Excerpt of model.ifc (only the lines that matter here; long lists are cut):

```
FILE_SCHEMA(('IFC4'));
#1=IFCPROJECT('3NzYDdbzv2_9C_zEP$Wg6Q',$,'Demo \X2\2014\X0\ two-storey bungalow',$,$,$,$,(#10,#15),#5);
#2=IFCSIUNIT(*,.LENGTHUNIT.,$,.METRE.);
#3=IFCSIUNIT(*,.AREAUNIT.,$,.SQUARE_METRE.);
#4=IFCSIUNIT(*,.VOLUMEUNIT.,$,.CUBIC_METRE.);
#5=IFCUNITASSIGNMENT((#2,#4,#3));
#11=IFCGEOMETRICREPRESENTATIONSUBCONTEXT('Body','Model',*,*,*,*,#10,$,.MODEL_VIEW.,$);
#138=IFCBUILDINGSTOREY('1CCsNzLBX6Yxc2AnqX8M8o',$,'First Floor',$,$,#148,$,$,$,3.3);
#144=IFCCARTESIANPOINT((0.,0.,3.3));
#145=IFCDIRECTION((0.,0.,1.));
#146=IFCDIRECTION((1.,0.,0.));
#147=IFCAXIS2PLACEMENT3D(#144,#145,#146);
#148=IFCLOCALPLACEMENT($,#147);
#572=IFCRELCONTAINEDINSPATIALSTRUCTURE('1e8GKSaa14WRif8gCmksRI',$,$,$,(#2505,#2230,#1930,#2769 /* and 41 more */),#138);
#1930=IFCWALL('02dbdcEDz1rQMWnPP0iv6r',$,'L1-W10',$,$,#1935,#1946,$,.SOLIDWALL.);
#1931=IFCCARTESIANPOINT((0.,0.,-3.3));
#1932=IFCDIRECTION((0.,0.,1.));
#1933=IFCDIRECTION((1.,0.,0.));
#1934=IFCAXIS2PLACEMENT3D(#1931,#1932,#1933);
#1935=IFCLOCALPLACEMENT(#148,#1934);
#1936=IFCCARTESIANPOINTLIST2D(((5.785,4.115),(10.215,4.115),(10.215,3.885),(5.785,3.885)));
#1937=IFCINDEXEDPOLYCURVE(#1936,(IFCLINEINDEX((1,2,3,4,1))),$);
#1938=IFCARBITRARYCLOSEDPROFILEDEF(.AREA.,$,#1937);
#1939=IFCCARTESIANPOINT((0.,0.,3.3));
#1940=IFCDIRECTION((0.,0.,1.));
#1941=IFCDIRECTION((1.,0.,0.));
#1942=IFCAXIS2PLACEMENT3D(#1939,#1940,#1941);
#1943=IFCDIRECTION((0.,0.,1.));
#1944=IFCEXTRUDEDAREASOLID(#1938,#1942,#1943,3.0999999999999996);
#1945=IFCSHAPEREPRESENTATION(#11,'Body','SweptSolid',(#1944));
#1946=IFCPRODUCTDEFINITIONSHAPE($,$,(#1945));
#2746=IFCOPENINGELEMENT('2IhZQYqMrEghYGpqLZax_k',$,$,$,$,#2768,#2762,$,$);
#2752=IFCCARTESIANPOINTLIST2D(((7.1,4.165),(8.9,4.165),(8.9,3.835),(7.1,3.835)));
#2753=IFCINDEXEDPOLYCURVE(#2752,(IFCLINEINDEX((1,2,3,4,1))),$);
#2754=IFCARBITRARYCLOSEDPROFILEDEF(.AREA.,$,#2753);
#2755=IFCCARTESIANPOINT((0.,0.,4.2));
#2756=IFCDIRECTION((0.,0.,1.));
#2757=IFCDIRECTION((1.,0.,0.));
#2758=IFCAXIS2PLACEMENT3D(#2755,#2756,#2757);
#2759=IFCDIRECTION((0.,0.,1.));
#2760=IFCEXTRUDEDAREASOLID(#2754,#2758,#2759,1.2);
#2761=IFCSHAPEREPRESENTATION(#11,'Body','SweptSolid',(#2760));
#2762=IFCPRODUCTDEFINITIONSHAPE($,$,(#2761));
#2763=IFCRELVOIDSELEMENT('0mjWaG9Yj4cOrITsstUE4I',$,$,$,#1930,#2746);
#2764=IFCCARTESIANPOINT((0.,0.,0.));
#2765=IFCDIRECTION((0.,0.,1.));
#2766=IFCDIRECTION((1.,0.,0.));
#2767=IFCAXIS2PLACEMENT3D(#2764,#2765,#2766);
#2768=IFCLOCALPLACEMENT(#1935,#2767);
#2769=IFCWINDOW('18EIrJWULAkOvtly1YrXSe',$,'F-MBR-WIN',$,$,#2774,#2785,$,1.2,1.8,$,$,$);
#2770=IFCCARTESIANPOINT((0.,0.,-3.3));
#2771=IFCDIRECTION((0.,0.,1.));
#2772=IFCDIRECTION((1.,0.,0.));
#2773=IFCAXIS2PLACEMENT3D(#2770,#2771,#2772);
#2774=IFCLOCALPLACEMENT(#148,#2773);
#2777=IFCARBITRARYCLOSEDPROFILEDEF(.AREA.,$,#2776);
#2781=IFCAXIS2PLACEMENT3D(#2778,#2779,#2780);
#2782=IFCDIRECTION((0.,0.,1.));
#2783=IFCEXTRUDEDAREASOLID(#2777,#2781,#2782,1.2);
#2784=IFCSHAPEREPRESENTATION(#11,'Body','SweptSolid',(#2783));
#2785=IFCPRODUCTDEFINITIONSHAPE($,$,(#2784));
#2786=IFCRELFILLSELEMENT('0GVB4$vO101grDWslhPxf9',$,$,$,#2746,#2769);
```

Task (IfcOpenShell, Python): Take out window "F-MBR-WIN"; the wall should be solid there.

```python
import ifcopenshell
import ifcopenshell.api.feature
import ifcopenshell.api.root
import ifcopenshell.geom
import ifcopenshell.util.shape

model = ifcopenshell.open("model.ifc")
settings = ifcopenshell.geom.settings()


def volume(element):
    """Net volume in cubic metres, openings subtracted."""
    shape = ifcopenshell.geom.create_shape(settings, element)
    return ifcopenshell.util.shape.get_volume(shape.geometry)


window = model.by_id(2769)
opening = window.FillsVoids[0].RelatingOpeningElement
wall = opening.VoidsElements[0].RelatingBuildingElement
before = volume(wall)

ifcopenshell.api.root.remove_product(model, product=window)
ifcopenshell.api.feature.remove_feature(model, feature=opening)

after = volume(wall)

print(f"wall volume {before:.3f} -> {after:.3f} m3")

model.write("model_edited.ifc")
```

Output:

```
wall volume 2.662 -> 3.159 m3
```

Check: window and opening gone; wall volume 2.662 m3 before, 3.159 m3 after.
